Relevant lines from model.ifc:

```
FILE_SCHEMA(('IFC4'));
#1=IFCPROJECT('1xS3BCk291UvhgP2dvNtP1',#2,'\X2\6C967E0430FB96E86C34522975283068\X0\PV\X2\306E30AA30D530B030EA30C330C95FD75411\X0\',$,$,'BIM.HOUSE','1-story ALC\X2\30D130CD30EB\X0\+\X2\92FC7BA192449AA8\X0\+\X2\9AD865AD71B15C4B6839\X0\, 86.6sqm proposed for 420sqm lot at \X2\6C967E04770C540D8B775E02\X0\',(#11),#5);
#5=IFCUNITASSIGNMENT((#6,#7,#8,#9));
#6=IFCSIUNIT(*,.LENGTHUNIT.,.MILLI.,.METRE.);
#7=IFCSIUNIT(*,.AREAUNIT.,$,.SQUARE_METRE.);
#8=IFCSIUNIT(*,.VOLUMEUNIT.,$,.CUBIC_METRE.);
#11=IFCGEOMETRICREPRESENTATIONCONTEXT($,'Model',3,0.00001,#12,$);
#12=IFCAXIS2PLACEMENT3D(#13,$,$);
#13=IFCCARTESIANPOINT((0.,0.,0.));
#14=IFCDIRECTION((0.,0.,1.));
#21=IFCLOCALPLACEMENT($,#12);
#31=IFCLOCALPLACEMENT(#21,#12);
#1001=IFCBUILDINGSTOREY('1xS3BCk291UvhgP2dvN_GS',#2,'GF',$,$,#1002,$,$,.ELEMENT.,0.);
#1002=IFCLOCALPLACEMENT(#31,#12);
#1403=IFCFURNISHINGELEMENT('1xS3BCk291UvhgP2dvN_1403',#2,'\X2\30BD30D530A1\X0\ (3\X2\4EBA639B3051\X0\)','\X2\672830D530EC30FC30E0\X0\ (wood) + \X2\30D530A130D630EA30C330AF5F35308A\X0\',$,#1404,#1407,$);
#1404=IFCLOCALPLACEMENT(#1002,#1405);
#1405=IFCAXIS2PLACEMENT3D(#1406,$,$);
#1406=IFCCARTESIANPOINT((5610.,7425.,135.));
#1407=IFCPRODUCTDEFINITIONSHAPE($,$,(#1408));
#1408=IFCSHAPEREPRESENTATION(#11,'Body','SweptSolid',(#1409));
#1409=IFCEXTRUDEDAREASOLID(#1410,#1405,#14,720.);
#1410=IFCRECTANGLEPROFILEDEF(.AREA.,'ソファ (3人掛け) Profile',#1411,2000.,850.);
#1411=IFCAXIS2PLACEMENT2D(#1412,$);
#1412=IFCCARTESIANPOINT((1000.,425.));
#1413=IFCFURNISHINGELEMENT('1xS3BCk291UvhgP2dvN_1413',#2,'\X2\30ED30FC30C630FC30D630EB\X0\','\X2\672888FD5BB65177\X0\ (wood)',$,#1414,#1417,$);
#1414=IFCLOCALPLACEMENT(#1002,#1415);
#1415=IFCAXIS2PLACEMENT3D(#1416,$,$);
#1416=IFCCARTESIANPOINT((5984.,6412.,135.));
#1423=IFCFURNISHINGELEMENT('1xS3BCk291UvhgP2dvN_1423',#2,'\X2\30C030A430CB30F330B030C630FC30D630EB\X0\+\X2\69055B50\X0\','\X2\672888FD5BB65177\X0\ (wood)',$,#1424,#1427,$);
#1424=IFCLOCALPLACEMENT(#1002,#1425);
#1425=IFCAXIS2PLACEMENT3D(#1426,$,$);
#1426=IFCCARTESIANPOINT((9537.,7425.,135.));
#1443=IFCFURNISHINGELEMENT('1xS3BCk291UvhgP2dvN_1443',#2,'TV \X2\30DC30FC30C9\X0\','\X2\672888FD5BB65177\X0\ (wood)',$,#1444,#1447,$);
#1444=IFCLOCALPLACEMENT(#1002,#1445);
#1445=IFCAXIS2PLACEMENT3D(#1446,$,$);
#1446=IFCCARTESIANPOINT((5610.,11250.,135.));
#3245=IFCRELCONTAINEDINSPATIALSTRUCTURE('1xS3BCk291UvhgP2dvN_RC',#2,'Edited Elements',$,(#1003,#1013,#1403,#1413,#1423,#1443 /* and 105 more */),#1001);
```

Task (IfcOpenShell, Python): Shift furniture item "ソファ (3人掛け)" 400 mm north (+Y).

```python
import ifcopenshell
import ifcopenshell.api.geometry
import ifcopenshell.util.placement
import ifcopenshell.util.unit

model = ifcopenshell.open("model.ifc")
unit_scale = ifcopenshell.util.unit.calculate_unit_scale(model)

item = model.by_guid("1xS3BCk291UvhgP2dvN_1403")
matrix = ifcopenshell.util.placement.get_local_placement(item.ObjectPlacement)
matrix[1, 3] += 0.4 / unit_scale
ifcopenshell.api.geometry.edit_object_placement(model, product=item, matrix=matrix, is_si=False)

print(ifcopenshell.util.placement.get_local_placement(item.ObjectPlacement).round(3) + 0.0)

model.write("model_rev.ifc")
```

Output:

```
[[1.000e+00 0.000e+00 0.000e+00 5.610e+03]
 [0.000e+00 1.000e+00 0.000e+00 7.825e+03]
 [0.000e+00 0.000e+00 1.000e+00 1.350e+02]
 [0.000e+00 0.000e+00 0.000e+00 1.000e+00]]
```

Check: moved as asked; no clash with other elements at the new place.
